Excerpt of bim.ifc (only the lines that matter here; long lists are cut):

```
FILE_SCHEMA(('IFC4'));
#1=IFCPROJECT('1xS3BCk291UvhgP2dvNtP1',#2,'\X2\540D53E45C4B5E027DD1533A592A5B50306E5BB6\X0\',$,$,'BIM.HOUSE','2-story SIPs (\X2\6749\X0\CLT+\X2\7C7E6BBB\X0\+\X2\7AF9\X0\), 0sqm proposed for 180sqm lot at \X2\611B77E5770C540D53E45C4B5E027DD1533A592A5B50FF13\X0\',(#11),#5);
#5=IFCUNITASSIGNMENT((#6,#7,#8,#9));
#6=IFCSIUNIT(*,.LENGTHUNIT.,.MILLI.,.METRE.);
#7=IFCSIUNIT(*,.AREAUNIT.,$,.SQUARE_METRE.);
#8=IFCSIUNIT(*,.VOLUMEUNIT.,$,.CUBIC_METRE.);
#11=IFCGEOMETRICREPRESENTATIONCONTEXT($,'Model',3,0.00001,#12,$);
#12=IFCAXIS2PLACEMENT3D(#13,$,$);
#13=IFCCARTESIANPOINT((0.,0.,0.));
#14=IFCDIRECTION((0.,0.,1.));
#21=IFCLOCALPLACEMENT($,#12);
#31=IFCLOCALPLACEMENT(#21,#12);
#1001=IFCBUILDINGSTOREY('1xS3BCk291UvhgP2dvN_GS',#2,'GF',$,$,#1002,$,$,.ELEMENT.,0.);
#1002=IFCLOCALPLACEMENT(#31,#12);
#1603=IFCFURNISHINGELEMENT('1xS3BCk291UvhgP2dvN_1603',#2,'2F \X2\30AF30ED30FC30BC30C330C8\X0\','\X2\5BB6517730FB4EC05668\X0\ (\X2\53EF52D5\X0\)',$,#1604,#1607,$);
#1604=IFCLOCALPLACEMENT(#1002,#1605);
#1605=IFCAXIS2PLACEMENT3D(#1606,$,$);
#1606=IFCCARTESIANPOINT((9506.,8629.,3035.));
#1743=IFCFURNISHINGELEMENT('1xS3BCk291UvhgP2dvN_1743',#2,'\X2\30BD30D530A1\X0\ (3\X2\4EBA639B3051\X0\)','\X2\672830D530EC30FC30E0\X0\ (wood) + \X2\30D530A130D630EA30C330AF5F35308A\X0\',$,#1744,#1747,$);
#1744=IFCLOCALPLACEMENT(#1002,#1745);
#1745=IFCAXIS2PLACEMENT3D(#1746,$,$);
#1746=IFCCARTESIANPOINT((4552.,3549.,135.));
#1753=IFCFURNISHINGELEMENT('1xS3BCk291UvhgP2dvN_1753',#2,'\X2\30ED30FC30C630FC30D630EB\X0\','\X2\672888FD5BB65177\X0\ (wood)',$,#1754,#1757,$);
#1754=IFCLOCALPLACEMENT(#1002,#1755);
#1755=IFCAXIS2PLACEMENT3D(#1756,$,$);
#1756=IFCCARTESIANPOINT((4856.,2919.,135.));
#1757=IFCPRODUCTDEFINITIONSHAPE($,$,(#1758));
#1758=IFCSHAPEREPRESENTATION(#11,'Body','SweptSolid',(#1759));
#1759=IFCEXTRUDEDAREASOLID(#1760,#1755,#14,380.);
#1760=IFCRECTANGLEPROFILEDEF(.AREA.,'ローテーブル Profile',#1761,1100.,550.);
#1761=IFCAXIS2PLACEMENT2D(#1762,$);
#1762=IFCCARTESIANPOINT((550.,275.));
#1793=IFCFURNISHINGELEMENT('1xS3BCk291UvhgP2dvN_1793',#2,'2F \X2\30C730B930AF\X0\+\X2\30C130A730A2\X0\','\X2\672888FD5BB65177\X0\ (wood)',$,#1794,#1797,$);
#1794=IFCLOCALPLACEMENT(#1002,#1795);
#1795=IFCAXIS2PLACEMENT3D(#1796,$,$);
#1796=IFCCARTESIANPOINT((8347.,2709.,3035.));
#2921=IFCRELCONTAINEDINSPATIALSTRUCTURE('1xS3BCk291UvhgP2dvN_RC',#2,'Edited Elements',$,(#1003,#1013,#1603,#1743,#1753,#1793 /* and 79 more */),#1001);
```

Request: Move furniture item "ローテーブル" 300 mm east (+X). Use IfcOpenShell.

```python
import ifcopenshell
import ifcopenshell.api.geometry
import ifcopenshell.util.placement

model = ifcopenshell.open("bim.ifc")

item = model.by_id(1753)
matrix = ifcopenshell.util.placement.get_local_placement(item.ObjectPlacement)
matrix[0, 3] += 300.0
ifcopenshell.api.geometry.edit_object_placement(model, product=item, matrix=matrix, is_si=False)

print(ifcopenshell.util.placement.get_local_placement(item.ObjectPlacement).round(3) + 0.0)

model.write("bim_v2.ifc")
```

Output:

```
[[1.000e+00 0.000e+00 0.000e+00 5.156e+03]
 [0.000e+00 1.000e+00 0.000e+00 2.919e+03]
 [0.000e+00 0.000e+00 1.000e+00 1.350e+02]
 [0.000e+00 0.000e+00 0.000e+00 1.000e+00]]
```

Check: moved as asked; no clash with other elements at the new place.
